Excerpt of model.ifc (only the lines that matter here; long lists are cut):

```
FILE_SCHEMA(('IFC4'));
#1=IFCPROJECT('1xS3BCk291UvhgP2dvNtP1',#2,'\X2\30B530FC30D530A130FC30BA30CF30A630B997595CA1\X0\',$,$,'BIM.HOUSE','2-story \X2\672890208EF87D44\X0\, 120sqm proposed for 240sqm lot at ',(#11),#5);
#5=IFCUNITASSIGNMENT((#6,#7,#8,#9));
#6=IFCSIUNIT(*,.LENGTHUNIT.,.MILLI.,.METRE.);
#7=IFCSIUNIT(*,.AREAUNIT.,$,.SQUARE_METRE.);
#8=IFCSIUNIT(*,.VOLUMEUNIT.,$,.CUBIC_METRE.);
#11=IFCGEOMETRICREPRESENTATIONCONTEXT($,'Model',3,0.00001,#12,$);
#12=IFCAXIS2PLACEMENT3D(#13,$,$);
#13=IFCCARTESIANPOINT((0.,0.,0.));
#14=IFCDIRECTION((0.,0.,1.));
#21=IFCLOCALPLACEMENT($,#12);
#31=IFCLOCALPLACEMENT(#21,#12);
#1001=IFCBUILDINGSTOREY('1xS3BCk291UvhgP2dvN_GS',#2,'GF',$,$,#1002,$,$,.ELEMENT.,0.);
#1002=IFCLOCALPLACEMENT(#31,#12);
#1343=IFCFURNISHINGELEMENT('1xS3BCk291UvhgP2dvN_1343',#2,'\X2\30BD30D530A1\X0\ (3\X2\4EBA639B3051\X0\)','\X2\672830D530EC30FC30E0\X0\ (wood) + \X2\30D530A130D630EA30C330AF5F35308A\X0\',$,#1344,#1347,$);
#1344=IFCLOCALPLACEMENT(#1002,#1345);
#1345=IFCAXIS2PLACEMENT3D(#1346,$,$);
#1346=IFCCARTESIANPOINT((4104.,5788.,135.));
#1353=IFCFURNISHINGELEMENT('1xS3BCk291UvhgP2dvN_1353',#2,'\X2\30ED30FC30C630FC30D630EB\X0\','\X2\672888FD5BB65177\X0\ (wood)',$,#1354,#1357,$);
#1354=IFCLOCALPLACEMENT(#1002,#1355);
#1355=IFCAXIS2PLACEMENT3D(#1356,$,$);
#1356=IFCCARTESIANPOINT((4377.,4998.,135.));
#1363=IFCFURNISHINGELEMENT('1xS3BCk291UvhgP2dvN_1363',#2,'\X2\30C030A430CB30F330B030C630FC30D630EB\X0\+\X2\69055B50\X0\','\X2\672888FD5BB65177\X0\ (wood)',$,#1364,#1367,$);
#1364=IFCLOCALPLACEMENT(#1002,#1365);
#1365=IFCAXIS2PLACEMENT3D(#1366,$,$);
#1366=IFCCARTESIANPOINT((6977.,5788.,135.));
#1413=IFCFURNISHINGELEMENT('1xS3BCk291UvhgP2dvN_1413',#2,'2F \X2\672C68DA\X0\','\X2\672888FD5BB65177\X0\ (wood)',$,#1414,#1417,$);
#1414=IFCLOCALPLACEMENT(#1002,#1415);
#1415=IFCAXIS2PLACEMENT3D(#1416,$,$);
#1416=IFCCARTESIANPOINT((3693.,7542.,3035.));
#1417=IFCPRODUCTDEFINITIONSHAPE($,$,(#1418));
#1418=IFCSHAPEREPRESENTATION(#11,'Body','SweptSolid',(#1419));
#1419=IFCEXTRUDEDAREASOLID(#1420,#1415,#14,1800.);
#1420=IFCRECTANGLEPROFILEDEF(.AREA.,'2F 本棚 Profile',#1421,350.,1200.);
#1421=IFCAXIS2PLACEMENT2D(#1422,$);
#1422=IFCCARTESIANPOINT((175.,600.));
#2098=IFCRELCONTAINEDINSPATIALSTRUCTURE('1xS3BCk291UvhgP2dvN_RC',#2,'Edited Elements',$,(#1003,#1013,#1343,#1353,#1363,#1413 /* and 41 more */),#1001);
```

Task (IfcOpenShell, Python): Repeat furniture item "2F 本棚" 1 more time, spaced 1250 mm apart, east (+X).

```python
import numpy as np
import ifcopenshell
import ifcopenshell.api.geometry
import ifcopenshell.api.root
import ifcopenshell.util.element
import ifcopenshell.util.placement

model = ifcopenshell.open("model.ifc")


def reuse_history(source, copy):
    """copy_class also copies each property set's owner history, people and application; keep the originals."""
    for rel in copy.IsDefinedBy:
        if rel.is_a("IfcRelDefinesByProperties") and (history := rel.RelatingPropertyDefinition.OwnerHistory):
            rel.RelatingPropertyDefinition.OwnerHistory = source.OwnerHistory
            ifcopenshell.util.element.remove_deep2(model, history)


source = model.by_id(1413)
base = ifcopenshell.util.placement.get_local_placement(source.ObjectPlacement)
step = np.array([1.0, 0.0, 0.0]) * 1250.0

for i in range(1, 2):
    copy = ifcopenshell.api.root.copy_class(model, product=source)
    copy.Representation = ifcopenshell.util.element.copy_deep(
        model, source.Representation, exclude=["IfcGeometricRepresentationContext", "IfcRepresentationMap"]
    )
    reuse_history(source, copy)
    matrix = base.copy()
    matrix[:3, 3] += i * step
    print("added at", matrix[:3, 3].round(3) + 0.0)
    ifcopenshell.api.geometry.edit_object_placement(model, product=copy, matrix=matrix, is_si=False)

model.write("model-out.ifc")
```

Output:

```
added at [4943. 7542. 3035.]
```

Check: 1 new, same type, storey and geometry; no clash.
